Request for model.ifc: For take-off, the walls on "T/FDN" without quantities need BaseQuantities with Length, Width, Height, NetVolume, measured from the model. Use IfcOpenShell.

First a look at what the model holds.

```python
import ifcopenshell
import ifcopenshell.util.element
import ifcopenshell.util.unit

model = ifcopenshell.open("model.ifc")
print(model.schema)
for unit_type in ("LENGTHUNIT", "AREAUNIT", "VOLUMEUNIT"):
    print(unit_type, ifcopenshell.util.unit.calculate_unit_scale(model, unit_type))
storey = next(s for s in model.by_type("IfcBuildingStorey") if s.Name == "T/FDN")
walls = [e for e in ifcopenshell.util.element.get_decomposition(storey) if e.is_a("IfcWall")]
for e in sorted(walls, key=lambda e: e.id()):
    print(e.id(), e.is_a(), e.Name, list(ifcopenshell.util.element.get_psets(e, qtos_only=True)), sep=" | ")
```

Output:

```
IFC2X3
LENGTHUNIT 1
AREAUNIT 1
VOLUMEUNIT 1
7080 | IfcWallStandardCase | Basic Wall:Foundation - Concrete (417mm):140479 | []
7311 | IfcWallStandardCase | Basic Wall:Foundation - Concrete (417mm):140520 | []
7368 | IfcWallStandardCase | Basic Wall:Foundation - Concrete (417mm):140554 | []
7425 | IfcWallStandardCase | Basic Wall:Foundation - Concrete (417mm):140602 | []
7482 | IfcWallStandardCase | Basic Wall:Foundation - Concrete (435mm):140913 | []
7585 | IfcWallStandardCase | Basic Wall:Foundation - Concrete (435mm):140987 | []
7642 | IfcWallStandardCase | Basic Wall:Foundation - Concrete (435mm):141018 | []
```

```python
import ifcopenshell
import ifcopenshell.api.pset
import ifcopenshell.geom
import ifcopenshell.util.element
import ifcopenshell.util.shape
import ifcopenshell.util.unit

model = ifcopenshell.open("model.ifc")
unit_scale = ifcopenshell.util.unit.calculate_unit_scale(model)
volume_scale = ifcopenshell.util.unit.calculate_unit_scale(model, "VOLUMEUNIT")
settings = ifcopenshell.geom.settings()

storey = next(s for s in model.by_type("IfcBuildingStorey") if s.Name == "T/FDN")
walls = [e for e in ifcopenshell.util.element.get_decomposition(storey) if e.is_a("IfcWall")]

for e in sorted(walls, key=lambda e: e.id()):
    if ifcopenshell.util.element.get_psets(e, qtos_only=True, should_inherit=False):
        continue
    # Geometry comes back in metres, in the element's own axes.
    shape = ifcopenshell.geom.create_shape(settings, e)
    values = {
        "Length": ifcopenshell.util.shape.get_x(shape.geometry) / unit_scale,
        "Width": ifcopenshell.util.shape.get_y(shape.geometry) / unit_scale,
        "Height": ifcopenshell.util.shape.get_z(shape.geometry) / unit_scale,
        "NetVolume": ifcopenshell.util.shape.get_volume(shape.geometry) / volume_scale,
    }
    qto = ifcopenshell.api.pset.add_qto(model, product=e, name="BaseQuantities")
    ifcopenshell.api.pset.edit_qto(model, qto=qto, properties=values)
    print(e.id(), {k: round(v, 3) for k, v in values.items()})

model.write("model_edited.ifc")
```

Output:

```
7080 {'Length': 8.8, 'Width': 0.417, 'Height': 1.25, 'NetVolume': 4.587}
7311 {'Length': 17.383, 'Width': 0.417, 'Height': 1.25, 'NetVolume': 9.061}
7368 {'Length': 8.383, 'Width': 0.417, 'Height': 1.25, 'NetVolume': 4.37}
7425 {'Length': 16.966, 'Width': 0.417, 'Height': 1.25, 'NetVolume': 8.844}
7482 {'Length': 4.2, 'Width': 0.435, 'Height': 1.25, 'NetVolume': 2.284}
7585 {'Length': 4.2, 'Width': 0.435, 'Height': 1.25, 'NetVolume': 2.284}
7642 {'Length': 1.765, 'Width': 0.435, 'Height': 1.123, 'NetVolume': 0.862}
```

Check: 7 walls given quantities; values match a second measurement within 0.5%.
